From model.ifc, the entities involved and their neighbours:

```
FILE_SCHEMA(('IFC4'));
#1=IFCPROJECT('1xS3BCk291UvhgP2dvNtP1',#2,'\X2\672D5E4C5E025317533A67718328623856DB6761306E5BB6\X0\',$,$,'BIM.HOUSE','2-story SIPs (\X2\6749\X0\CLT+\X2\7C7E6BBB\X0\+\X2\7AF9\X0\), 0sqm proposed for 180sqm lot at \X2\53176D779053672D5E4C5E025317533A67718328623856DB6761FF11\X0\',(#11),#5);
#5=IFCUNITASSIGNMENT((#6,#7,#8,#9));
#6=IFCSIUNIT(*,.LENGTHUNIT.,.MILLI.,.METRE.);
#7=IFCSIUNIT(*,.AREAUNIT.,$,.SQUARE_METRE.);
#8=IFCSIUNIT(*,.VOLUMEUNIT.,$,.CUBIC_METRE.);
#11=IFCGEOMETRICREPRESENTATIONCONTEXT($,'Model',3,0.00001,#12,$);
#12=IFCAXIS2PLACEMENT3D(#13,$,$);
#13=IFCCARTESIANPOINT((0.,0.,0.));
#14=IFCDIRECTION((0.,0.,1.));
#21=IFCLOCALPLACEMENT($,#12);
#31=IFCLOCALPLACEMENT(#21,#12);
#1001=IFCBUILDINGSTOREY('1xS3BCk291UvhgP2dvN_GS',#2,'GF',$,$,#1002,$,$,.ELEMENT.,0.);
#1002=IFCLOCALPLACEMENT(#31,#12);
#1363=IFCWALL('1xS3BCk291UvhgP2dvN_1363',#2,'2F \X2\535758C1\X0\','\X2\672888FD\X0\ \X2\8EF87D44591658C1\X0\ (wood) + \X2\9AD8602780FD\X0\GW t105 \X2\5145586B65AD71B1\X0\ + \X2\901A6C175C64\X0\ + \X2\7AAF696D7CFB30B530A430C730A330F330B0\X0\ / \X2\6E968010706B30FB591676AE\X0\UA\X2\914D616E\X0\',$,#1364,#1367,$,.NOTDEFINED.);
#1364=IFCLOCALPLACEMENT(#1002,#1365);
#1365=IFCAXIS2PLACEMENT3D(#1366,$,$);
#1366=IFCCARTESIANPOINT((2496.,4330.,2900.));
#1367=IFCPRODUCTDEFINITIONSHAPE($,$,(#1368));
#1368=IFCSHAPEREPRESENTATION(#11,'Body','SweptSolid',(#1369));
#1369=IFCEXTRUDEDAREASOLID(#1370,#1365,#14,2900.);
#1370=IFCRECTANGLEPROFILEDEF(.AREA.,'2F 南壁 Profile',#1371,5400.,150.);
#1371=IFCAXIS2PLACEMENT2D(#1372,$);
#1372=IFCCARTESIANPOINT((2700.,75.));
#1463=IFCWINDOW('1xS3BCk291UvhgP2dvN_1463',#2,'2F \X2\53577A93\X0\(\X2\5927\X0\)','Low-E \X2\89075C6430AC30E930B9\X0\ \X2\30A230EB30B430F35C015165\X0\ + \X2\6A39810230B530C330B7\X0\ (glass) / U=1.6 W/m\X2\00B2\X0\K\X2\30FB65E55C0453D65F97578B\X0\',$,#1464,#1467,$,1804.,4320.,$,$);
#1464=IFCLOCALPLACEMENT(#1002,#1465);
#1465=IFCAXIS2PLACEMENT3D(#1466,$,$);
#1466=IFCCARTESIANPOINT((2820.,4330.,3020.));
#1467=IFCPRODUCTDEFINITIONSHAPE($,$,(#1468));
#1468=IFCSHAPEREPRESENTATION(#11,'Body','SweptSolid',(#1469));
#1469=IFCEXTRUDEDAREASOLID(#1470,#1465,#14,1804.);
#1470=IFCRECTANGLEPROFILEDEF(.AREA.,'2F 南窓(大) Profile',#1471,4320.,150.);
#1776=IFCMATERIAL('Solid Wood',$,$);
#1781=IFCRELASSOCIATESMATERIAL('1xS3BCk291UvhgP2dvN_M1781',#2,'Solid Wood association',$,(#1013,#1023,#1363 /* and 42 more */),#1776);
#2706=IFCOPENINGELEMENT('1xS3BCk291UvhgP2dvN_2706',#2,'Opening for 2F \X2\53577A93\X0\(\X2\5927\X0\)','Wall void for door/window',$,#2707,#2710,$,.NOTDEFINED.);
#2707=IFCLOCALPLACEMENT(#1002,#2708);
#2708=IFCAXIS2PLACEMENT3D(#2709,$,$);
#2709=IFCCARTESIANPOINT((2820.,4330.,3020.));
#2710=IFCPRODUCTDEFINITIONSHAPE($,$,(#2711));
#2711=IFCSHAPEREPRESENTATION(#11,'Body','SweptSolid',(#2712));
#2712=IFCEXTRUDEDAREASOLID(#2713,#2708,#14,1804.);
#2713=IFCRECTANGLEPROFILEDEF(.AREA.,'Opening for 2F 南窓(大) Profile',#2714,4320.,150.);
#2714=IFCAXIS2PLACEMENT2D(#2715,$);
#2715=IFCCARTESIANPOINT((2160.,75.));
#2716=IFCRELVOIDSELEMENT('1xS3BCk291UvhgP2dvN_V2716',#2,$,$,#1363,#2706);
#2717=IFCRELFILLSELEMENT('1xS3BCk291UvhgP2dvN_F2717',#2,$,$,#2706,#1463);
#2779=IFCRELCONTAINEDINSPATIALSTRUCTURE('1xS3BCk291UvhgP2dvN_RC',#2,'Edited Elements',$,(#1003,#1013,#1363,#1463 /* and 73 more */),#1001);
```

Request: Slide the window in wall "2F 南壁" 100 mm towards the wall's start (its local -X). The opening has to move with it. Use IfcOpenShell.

```python
import ifcopenshell
import ifcopenshell.api.geometry
import ifcopenshell.util.placement
import ifcopenshell.util.unit

model = ifcopenshell.open("model.ifc")
unit_scale = ifcopenshell.util.unit.calculate_unit_scale(model)

window = model.by_guid("1xS3BCk291UvhgP2dvN_1463")
opening = window.FillsVoids[0].RelatingOpeningElement
wall = opening.VoidsElements[0].RelatingBuildingElement

wall_matrix = ifcopenshell.util.placement.get_local_placement(wall.ObjectPlacement)
shift = wall_matrix[:3, 0] * -0.1 / unit_scale
before = ifcopenshell.util.placement.get_local_placement(window.ObjectPlacement)[:3, 3].copy()

# The window is not placed relative to its opening, so move both.
for product in (opening, window):
    matrix = ifcopenshell.util.placement.get_local_placement(product.ObjectPlacement)
    matrix[:3, 3] += shift
    ifcopenshell.api.geometry.edit_object_placement(model, product=product, matrix=matrix, is_si=False)

after = ifcopenshell.util.placement.get_local_placement(window.ObjectPlacement)[:3, 3]
print("window moved by", (after - before).round(3) + 0.0)

model.write("model-out.ifc")
```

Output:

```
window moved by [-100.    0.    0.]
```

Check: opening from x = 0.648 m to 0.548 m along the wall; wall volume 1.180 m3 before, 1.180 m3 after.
